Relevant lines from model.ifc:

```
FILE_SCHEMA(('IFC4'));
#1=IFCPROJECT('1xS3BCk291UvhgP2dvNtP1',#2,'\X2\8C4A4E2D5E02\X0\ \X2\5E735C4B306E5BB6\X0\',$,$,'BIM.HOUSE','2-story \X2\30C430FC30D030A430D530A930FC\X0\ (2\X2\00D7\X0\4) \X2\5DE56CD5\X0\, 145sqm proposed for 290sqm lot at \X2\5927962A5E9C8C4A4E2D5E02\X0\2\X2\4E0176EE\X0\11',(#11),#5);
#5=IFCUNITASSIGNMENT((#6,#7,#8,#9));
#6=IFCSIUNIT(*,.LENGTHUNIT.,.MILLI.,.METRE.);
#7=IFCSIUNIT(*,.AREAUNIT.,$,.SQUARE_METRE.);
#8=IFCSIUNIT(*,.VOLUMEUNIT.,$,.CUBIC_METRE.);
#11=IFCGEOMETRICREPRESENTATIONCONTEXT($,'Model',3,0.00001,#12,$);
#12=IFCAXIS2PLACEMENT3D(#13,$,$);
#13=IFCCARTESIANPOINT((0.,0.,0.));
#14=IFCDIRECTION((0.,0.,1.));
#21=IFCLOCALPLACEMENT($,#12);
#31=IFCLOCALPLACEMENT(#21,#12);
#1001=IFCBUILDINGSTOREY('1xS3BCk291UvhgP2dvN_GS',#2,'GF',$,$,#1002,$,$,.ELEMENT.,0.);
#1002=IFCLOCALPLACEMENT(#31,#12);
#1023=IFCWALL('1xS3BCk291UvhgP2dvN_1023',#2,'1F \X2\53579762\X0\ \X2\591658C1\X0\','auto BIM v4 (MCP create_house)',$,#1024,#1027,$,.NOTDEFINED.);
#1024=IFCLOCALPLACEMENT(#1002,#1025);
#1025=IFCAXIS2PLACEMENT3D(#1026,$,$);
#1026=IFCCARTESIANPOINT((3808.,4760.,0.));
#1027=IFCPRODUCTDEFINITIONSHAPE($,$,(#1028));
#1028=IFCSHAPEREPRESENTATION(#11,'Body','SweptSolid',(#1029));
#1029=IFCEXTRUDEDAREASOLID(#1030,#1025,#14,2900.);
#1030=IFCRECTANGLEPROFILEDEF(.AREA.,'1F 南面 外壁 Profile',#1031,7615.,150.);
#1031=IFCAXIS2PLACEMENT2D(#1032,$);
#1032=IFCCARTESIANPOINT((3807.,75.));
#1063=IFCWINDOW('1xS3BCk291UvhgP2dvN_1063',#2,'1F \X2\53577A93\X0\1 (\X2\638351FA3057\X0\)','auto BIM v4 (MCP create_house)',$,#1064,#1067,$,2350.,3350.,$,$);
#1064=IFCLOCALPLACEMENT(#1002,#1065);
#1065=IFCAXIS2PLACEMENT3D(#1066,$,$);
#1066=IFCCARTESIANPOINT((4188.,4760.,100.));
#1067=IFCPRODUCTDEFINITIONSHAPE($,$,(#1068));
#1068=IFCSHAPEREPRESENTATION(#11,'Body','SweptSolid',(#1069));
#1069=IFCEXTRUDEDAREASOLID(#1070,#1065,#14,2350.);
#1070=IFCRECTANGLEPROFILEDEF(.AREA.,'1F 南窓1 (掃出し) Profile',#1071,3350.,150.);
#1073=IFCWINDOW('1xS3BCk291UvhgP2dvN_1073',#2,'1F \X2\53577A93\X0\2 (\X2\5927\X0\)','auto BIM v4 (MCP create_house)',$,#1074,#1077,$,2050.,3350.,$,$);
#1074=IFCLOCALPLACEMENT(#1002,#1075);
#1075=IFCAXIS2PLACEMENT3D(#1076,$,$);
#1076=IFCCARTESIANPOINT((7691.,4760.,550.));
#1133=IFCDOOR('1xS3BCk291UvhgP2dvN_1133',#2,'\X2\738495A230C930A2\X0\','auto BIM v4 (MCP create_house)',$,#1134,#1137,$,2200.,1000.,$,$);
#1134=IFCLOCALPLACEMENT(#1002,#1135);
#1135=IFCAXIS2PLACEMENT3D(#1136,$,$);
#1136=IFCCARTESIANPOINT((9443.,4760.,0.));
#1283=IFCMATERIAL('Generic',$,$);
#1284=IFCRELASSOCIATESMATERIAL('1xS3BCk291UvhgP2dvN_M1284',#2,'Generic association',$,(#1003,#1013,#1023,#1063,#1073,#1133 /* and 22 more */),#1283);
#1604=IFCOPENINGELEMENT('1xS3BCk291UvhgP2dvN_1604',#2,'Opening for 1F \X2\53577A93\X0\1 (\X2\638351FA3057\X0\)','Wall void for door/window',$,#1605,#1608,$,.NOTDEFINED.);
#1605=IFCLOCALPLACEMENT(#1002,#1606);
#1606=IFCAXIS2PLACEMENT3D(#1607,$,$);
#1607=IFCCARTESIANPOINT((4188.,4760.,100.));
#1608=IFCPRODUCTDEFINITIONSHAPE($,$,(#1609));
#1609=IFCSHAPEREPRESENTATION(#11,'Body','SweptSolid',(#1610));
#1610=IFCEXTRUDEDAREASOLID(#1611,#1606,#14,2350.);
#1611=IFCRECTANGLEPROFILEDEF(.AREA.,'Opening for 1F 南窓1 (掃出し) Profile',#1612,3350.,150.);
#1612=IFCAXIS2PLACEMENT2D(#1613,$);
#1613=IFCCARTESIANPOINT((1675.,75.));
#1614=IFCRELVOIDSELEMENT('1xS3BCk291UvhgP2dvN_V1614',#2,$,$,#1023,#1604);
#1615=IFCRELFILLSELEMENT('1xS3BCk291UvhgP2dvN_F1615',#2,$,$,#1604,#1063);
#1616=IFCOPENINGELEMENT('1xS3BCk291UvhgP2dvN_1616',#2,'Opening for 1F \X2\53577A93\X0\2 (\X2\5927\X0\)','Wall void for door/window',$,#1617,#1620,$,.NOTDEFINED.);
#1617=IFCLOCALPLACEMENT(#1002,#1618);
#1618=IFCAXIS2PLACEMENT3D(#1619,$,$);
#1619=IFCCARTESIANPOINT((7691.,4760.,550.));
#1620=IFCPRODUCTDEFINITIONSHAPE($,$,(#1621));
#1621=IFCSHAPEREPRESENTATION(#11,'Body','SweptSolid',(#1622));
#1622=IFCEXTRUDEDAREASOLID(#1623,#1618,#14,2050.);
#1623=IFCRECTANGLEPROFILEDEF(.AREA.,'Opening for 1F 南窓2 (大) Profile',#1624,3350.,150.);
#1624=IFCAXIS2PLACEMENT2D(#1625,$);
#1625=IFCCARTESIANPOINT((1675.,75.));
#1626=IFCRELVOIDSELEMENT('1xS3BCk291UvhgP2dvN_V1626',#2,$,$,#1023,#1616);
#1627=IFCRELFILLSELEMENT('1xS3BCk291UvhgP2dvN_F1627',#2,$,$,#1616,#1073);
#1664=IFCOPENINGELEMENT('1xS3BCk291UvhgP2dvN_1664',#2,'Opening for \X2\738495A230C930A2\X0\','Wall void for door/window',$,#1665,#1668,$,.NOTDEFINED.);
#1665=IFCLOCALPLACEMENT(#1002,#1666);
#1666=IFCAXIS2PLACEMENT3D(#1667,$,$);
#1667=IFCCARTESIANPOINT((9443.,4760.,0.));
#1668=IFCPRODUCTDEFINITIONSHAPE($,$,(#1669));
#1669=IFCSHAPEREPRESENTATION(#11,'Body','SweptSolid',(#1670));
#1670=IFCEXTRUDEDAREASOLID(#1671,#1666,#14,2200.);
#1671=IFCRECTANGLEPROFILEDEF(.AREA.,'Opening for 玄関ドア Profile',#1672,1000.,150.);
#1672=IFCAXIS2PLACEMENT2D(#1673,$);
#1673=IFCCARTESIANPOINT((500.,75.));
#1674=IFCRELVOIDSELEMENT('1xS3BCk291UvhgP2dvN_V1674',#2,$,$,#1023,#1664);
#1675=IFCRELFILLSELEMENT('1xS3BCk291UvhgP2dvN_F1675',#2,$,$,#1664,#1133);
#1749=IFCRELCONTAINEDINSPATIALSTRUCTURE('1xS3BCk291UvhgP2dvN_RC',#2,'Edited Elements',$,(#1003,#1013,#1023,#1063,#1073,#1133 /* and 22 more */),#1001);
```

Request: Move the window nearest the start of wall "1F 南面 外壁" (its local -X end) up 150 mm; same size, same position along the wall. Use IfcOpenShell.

```python
import numpy as np
import ifcopenshell
import ifcopenshell.api.geometry
import ifcopenshell.util.placement
import ifcopenshell.util.unit

model = ifcopenshell.open("model.ifc")
unit_scale = ifcopenshell.util.unit.calculate_unit_scale(model)

window = model.by_id(1063)
opening = window.FillsVoids[0].RelatingOpeningElement
dz = 0.15 / unit_scale

shift = np.array([0.0, 0.0, dz])
# The window is not placed relative to its opening, so move both.
for product in (opening, window):
    matrix = ifcopenshell.util.placement.get_local_placement(product.ObjectPlacement)
    matrix[:3, 3] += shift
    ifcopenshell.api.geometry.edit_object_placement(model, product=product, matrix=matrix, is_si=False)

print(f"moved by {dz * unit_scale:+.3f} m")

model.write("model_updated.ifc")
```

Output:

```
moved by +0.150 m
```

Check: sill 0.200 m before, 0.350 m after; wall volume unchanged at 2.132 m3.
